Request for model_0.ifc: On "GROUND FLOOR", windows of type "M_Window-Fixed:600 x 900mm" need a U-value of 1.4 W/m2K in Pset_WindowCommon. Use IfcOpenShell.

First a look at what the model holds.

```python
import ifcopenshell
import ifcopenshell.util.element

model = ifcopenshell.open("model_0.ifc")
print(model.schema)
storey = next(s for s in model.by_type("IfcBuildingStorey") if s.Name == "GROUND FLOOR")
windows = [e for e in ifcopenshell.util.element.get_decomposition(storey) if e.is_a("IfcWindow")]
seen = {}
for e in windows:
    element_type = ifcopenshell.util.element.get_type(e)
    key = (element_type.Name if element_type != e and element_type else None, ifcopenshell.util.element.get_pset(e, "Pset_WindowCommon", "ThermalTransmittance"))
    seen[key] = seen.get(key, 0) + 1
for (name, value), count in sorted(seen.items(), key=str):
    print(count, "x", name, "|", value)
```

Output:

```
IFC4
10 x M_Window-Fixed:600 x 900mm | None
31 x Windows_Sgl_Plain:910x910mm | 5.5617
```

```python
import ifcopenshell
import ifcopenshell.api.pset
import ifcopenshell.util.element

model = ifcopenshell.open("model_0.ifc")

storey = next(s for s in model.by_type("IfcBuildingStorey") if s.Name == "GROUND FLOOR")
windows = [e for e in ifcopenshell.util.element.get_decomposition(storey) if e.is_a("IfcWindow")]

count = 0
for e in windows:
    element_type = ifcopenshell.util.element.get_type(e)
    if element_type in (None, e) or element_type.Name != "M_Window-Fixed:600 x 900mm":
        continue
    # add_pset returns the element's existing set when there is one.
    pset = ifcopenshell.api.pset.add_pset(model, product=e, name="Pset_WindowCommon")
    ifcopenshell.api.pset.edit_pset(model, pset=pset, properties={"ThermalTransmittance": 1.4})
    count += 1

print(count, "windows updated")

model.write("model_0_updated.ifc")
```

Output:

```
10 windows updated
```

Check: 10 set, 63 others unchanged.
